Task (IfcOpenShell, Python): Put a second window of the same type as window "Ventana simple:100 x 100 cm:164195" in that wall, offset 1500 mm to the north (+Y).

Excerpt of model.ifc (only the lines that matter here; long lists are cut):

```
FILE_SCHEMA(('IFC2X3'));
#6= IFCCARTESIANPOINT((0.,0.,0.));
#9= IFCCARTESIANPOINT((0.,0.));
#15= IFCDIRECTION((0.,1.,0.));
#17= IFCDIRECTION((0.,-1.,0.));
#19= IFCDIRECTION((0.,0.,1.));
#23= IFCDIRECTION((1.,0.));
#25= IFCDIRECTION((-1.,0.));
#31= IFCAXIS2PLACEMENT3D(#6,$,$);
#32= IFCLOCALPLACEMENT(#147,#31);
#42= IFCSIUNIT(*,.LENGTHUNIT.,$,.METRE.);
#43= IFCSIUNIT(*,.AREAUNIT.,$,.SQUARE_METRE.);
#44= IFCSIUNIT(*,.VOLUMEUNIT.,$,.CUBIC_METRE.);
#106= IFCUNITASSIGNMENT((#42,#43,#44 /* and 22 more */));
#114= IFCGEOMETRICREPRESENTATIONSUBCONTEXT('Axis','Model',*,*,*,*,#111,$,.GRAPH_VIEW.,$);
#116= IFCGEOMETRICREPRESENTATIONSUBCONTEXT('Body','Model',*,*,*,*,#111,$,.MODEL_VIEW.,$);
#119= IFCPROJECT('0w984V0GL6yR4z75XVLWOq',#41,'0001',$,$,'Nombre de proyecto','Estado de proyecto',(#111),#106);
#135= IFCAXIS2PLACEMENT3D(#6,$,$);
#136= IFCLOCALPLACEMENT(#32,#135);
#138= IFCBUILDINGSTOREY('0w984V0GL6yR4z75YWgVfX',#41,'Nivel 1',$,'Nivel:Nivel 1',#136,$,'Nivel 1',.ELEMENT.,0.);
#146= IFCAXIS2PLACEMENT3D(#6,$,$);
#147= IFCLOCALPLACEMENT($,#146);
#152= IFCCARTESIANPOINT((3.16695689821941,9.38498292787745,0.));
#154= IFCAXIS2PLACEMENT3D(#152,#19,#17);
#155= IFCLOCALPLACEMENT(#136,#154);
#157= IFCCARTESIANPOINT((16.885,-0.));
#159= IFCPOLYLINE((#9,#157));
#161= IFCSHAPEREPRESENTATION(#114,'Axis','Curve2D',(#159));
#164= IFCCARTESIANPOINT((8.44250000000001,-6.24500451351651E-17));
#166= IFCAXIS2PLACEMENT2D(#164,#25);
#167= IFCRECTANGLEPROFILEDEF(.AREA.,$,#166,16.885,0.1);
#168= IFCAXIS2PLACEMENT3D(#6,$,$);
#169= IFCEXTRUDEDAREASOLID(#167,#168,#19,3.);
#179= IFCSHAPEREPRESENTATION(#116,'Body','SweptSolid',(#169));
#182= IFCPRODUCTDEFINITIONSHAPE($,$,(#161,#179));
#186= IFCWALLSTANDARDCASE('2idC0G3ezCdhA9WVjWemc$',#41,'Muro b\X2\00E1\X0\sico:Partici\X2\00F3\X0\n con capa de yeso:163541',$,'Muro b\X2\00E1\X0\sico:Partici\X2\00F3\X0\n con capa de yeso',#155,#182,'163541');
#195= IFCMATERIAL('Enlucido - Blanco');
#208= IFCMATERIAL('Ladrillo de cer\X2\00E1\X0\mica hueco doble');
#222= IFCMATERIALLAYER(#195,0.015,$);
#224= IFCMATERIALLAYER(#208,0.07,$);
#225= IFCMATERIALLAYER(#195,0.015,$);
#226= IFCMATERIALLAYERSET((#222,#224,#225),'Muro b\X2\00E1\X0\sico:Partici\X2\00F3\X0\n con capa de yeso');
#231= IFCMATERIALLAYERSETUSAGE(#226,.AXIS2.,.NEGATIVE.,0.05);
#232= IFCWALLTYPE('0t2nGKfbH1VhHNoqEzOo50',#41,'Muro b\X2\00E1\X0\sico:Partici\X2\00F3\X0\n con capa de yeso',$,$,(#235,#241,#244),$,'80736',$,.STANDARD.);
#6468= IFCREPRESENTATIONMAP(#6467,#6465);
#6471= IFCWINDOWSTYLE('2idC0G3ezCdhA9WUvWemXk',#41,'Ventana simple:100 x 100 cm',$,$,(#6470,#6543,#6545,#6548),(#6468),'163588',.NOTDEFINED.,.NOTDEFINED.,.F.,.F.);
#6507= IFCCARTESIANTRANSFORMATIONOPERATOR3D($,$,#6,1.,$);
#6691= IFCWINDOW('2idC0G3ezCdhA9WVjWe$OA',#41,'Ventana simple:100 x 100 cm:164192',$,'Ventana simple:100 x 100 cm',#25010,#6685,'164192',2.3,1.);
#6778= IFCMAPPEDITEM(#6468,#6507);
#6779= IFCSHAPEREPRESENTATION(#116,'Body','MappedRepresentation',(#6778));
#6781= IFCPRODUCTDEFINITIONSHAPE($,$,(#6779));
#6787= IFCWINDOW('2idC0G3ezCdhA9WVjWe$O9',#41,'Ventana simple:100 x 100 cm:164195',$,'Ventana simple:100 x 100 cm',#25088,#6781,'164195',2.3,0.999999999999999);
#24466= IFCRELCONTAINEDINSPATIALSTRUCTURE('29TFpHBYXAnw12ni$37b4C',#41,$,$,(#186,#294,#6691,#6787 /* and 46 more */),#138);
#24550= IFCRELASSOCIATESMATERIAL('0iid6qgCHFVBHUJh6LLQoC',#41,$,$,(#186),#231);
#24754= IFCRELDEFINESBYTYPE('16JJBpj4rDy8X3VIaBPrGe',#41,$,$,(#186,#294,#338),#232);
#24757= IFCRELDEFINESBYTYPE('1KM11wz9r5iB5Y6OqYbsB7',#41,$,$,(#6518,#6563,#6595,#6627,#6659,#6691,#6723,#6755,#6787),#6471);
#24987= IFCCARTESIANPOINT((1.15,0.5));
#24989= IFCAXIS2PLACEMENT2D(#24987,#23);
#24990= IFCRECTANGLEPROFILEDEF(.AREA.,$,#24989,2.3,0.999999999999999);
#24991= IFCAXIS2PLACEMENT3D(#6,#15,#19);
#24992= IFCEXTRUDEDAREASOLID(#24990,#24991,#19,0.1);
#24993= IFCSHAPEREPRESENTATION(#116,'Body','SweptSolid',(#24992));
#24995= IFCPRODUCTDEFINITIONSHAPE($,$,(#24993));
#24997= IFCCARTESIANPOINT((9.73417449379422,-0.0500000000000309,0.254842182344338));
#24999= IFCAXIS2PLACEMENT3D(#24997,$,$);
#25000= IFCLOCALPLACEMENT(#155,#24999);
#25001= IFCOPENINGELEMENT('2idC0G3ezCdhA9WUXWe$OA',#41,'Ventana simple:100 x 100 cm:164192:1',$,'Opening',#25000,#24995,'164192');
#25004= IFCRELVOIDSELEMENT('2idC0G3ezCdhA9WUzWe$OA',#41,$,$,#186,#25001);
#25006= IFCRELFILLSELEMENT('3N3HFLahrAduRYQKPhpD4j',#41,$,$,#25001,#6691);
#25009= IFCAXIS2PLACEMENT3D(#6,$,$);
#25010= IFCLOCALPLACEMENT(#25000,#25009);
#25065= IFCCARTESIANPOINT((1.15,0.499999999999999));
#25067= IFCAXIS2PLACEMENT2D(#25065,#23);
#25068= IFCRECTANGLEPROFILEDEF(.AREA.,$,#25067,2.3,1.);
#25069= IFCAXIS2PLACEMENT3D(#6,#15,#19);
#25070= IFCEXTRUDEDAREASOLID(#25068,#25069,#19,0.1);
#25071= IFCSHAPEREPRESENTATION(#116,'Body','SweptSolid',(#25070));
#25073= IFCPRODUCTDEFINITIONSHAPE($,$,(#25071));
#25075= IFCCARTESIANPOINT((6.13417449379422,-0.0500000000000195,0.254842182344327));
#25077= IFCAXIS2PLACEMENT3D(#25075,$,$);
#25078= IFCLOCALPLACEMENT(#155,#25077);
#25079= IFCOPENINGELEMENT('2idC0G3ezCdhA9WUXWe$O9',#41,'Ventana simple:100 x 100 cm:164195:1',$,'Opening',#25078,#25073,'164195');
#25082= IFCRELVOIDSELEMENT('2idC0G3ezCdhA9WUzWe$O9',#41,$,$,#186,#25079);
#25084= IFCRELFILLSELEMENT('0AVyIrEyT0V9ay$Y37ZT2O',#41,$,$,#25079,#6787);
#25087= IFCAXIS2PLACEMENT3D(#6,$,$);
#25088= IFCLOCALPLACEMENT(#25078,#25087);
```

```python
import ifcopenshell
import ifcopenshell.api.feature
import ifcopenshell.api.geometry
import ifcopenshell.api.root
import ifcopenshell.geom
import ifcopenshell.util.element
import ifcopenshell.util.placement
import ifcopenshell.util.shape
import ifcopenshell.util.unit

model = ifcopenshell.open("model.ifc")
unit_scale = ifcopenshell.util.unit.calculate_unit_scale(model)
settings = ifcopenshell.geom.settings()


def volume(element):
    """Net volume in cubic metres, openings subtracted."""
    shape = ifcopenshell.geom.create_shape(settings, element)
    return ifcopenshell.util.shape.get_volume(shape.geometry)


def reuse_history(source, copy):
    """copy_class also copies each property set's owner history, people and application; keep the originals."""
    for rel in copy.IsDefinedBy:
        if rel.is_a("IfcRelDefinesByProperties") and (history := rel.RelatingPropertyDefinition.OwnerHistory):
            rel.RelatingPropertyDefinition.OwnerHistory = source.OwnerHistory
            ifcopenshell.util.element.remove_deep2(model, history)


window = model.by_id(6787)
opening = window.FillsVoids[0].RelatingOpeningElement
wall = opening.VoidsElements[0].RelatingBuildingElement
before = volume(wall)
shift = ifcopenshell.util.placement.get_local_placement(wall.ObjectPlacement)[:3, 0] * -1.5 / unit_scale

# copy_class copies the void relationship, type, container and properties, but no geometry.
new_opening = ifcopenshell.api.root.copy_class(model, product=opening)
new_opening.Representation = ifcopenshell.util.element.copy_deep(
    model, opening.Representation, exclude=["IfcGeometricRepresentationContext", "IfcRepresentationMap"]
)
new_opening.Name = "Ventana simple:100 x 100 cm"
new_opening.Tag = None
new_window = ifcopenshell.api.root.copy_class(model, product=window)
new_window.Representation = ifcopenshell.util.element.copy_deep(
    model, window.Representation, exclude=["IfcGeometricRepresentationContext", "IfcRepresentationMap"]
)
new_window.Name = "Ventana simple:100 x 100 cm"
new_window.Tag = None
reuse_history(window, new_window)
fills = ifcopenshell.api.feature.add_filling(model, opening=new_opening, element=new_window)
fills.OwnerHistory = new_window.OwnerHistory  # required in IFC2X3

for old, new in ((opening, new_opening), (window, new_window)):
    matrix = ifcopenshell.util.placement.get_local_placement(old.ObjectPlacement)
    matrix[:3, 3] += shift
    ifcopenshell.api.geometry.edit_object_placement(model, product=new, matrix=matrix, is_si=False)

after = volume(wall)

print(f"wall volume {before:.3f} -> {after:.3f} m3")

model.write("model_edited.ifc")
```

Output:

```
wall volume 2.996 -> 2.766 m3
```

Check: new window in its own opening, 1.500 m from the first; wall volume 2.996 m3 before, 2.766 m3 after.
